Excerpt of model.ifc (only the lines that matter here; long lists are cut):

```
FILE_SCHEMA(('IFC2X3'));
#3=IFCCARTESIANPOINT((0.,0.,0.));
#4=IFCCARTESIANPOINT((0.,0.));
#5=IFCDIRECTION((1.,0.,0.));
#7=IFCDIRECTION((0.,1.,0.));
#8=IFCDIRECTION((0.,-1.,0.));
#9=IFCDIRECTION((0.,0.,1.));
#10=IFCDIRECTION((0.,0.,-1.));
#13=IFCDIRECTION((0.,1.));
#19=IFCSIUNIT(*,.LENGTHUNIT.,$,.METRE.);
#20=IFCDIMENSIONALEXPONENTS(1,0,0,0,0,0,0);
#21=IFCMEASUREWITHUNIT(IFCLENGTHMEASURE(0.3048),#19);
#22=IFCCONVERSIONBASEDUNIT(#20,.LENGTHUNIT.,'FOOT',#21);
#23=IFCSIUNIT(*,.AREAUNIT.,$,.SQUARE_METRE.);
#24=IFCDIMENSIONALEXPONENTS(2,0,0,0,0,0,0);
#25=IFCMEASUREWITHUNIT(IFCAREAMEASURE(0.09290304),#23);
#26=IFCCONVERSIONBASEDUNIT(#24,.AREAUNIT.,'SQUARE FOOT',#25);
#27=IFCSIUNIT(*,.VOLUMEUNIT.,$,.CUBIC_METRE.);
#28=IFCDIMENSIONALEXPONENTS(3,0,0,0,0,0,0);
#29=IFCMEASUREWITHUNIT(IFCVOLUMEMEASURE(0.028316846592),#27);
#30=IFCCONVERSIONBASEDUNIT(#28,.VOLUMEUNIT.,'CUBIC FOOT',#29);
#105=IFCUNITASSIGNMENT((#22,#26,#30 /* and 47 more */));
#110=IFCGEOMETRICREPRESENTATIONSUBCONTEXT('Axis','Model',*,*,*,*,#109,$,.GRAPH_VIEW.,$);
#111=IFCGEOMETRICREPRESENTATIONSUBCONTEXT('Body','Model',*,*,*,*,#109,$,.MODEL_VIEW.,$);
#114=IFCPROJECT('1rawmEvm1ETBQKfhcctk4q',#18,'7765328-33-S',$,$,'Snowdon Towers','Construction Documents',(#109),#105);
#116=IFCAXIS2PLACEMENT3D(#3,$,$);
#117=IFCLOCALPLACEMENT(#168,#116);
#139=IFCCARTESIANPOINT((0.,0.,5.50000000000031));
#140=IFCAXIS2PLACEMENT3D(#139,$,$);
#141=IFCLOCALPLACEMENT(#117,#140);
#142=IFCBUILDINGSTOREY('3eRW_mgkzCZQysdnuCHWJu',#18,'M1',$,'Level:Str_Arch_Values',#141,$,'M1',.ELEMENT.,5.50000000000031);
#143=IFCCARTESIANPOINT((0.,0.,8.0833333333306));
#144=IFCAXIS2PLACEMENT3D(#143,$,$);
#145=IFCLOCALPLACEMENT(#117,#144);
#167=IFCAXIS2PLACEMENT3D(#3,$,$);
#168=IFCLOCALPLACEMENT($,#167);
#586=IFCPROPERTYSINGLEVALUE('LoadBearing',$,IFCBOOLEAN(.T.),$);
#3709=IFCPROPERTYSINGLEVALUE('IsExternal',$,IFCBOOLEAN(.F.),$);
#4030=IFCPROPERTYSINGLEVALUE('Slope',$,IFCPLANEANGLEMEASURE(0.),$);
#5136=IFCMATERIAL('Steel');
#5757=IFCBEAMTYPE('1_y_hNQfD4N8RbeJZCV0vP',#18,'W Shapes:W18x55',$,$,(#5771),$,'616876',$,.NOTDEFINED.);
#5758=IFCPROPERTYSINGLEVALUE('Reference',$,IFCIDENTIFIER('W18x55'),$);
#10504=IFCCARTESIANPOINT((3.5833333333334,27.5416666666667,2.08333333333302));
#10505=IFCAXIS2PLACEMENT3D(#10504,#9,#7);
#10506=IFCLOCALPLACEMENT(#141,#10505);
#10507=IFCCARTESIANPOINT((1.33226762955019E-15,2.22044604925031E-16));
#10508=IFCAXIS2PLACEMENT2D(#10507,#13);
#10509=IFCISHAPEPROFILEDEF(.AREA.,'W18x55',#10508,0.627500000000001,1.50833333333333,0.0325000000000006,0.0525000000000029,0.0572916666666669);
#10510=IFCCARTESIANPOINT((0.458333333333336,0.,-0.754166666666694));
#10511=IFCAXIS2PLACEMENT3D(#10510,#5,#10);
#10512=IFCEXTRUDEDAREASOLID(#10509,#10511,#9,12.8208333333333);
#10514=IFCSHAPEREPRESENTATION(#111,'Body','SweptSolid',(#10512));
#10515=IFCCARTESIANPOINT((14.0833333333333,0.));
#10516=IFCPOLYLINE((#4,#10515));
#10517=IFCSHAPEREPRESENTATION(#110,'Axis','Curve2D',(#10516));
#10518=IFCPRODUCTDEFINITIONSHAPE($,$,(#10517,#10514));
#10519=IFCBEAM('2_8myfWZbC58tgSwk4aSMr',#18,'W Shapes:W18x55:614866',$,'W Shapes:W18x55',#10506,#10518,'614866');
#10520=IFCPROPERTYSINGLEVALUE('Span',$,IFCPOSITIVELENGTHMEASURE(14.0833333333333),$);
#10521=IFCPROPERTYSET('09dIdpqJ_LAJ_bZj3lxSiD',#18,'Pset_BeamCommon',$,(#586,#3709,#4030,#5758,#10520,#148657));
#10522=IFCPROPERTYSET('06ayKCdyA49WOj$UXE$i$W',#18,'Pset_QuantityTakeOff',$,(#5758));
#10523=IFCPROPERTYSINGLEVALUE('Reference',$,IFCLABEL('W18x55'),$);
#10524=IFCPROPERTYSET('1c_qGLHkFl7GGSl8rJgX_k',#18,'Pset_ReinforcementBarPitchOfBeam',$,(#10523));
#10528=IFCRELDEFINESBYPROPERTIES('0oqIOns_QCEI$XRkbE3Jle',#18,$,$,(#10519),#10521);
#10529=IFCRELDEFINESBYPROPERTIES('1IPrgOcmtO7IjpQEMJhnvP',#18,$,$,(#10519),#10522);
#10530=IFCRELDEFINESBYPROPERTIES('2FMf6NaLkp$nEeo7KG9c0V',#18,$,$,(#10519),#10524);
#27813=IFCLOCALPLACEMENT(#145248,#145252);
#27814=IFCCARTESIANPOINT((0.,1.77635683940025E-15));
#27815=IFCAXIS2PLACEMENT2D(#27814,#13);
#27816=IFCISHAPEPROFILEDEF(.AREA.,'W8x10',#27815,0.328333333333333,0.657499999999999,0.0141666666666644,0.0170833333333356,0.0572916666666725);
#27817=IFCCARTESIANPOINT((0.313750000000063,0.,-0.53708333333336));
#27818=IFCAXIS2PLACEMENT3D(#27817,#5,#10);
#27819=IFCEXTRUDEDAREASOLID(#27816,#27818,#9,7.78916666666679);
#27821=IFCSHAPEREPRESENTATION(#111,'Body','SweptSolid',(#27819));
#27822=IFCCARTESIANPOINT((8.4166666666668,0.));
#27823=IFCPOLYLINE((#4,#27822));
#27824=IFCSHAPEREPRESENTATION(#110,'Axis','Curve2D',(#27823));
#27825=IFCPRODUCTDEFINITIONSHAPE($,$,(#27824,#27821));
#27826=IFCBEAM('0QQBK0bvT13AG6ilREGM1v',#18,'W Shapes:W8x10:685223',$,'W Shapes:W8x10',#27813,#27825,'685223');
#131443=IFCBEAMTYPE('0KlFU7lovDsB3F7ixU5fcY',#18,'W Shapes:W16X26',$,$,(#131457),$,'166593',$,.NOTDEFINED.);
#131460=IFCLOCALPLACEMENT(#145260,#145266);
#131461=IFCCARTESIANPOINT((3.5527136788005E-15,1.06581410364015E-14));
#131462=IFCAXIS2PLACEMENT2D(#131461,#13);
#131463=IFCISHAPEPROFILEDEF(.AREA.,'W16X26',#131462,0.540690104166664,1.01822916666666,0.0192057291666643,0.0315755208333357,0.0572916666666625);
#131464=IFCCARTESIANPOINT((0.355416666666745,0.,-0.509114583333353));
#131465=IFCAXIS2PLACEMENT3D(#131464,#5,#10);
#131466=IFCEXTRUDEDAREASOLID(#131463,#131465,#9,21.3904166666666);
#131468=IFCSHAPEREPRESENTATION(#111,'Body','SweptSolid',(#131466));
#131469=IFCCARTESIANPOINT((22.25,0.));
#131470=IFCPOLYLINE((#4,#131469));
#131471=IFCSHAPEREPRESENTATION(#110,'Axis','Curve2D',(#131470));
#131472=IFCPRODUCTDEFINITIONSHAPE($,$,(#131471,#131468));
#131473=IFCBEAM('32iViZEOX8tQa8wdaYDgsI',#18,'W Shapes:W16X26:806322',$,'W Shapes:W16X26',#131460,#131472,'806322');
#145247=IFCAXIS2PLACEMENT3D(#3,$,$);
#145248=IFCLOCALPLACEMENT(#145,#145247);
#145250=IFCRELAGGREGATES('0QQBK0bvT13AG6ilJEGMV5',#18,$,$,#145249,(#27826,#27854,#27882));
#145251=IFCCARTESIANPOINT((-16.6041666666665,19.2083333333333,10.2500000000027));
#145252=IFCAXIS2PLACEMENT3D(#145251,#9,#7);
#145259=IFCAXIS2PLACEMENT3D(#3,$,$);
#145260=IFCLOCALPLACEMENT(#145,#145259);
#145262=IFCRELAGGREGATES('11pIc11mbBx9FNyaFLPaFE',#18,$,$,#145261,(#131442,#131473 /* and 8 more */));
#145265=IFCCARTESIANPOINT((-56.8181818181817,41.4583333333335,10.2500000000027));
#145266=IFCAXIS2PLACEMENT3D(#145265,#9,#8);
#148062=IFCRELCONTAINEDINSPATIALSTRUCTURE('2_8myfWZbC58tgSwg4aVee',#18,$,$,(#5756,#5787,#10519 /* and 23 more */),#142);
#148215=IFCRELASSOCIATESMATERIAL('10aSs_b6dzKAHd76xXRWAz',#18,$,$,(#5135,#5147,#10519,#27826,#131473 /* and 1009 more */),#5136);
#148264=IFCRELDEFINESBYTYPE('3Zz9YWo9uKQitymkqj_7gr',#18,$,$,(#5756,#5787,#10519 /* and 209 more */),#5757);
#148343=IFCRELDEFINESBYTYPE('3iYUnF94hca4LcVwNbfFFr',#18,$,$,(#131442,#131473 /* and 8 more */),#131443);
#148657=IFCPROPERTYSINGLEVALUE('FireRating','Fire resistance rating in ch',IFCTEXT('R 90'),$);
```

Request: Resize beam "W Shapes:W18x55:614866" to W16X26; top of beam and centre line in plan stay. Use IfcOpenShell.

```python
import ifcopenshell
import ifcopenshell.api.pset
import ifcopenshell.api.type
import ifcopenshell.util.element
import ifcopenshell.util.representation

model = ifcopenshell.open("model.ifc")

member = model.by_guid("2_8myfWZbC58tgSwk4aSMr")
source = next(p for p in model.by_type("IfcIShapeProfileDef") if p.ProfileName == "W16X26")

body = ifcopenshell.util.representation.get_representation(member, "Model", "Body")
solid = body.Items[0]
old_profile = solid.SweptArea

# Copy the section's sizes but keep this member's own profile position.
profile = ifcopenshell.util.element.copy(model, source)
# Profiles are centred, so shift by half the change in depth to hold the top.
shift = (old_profile.OverallDepth - profile.OverallDepth) / 2
x, y = old_profile.Position.Location.Coordinates
up = (-1.0, 0.0)  # upwards, in the solid's own plane
location = model.createIfcCartesianPoint((x + up[0] * shift, y + up[1] * shift))
profile.Position = model.createIfcAxis2Placement2D(location, old_profile.Position.RefDirection)
solid.SweptArea = profile
if not model.get_total_inverses(old_profile):
    ifcopenshell.util.element.remove_deep2(model, old_profile)

new_type = model.by_guid("0KlFU7lovDsB3F7ixU5fcY")
ifcopenshell.api.type.assign_type(
    model, related_objects=[member], relating_type=new_type, should_map_representations=False
)
member.Name = member.Name.replace("W18x55", "W16X26")
member.ObjectType = "W Shapes:W16X26"
pset = model.by_id(ifcopenshell.util.element.get_pset(member, "Pset_BeamCommon", should_inherit=False)["id"])
ifcopenshell.api.pset.edit_pset(model, pset=pset, properties={"Reference": "W16X26"})
pset = model.by_id(ifcopenshell.util.element.get_pset(member, "Pset_QuantityTakeOff", should_inherit=False)["id"])
ifcopenshell.api.pset.edit_pset(model, pset=pset, properties={"Reference": "W16X26"})
pset = model.by_id(ifcopenshell.util.element.get_pset(member, "Pset_ReinforcementBarPitchOfBeam", should_inherit=False)["id"])
ifcopenshell.api.pset.edit_pset(model, pset=pset, properties={"Reference": "W16X26"})

print(solid.SweptArea)

model.write("model_rev.ifc")
```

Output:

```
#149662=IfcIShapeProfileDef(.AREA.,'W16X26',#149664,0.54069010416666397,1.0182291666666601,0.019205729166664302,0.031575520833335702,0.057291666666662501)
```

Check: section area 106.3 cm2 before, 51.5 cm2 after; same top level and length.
